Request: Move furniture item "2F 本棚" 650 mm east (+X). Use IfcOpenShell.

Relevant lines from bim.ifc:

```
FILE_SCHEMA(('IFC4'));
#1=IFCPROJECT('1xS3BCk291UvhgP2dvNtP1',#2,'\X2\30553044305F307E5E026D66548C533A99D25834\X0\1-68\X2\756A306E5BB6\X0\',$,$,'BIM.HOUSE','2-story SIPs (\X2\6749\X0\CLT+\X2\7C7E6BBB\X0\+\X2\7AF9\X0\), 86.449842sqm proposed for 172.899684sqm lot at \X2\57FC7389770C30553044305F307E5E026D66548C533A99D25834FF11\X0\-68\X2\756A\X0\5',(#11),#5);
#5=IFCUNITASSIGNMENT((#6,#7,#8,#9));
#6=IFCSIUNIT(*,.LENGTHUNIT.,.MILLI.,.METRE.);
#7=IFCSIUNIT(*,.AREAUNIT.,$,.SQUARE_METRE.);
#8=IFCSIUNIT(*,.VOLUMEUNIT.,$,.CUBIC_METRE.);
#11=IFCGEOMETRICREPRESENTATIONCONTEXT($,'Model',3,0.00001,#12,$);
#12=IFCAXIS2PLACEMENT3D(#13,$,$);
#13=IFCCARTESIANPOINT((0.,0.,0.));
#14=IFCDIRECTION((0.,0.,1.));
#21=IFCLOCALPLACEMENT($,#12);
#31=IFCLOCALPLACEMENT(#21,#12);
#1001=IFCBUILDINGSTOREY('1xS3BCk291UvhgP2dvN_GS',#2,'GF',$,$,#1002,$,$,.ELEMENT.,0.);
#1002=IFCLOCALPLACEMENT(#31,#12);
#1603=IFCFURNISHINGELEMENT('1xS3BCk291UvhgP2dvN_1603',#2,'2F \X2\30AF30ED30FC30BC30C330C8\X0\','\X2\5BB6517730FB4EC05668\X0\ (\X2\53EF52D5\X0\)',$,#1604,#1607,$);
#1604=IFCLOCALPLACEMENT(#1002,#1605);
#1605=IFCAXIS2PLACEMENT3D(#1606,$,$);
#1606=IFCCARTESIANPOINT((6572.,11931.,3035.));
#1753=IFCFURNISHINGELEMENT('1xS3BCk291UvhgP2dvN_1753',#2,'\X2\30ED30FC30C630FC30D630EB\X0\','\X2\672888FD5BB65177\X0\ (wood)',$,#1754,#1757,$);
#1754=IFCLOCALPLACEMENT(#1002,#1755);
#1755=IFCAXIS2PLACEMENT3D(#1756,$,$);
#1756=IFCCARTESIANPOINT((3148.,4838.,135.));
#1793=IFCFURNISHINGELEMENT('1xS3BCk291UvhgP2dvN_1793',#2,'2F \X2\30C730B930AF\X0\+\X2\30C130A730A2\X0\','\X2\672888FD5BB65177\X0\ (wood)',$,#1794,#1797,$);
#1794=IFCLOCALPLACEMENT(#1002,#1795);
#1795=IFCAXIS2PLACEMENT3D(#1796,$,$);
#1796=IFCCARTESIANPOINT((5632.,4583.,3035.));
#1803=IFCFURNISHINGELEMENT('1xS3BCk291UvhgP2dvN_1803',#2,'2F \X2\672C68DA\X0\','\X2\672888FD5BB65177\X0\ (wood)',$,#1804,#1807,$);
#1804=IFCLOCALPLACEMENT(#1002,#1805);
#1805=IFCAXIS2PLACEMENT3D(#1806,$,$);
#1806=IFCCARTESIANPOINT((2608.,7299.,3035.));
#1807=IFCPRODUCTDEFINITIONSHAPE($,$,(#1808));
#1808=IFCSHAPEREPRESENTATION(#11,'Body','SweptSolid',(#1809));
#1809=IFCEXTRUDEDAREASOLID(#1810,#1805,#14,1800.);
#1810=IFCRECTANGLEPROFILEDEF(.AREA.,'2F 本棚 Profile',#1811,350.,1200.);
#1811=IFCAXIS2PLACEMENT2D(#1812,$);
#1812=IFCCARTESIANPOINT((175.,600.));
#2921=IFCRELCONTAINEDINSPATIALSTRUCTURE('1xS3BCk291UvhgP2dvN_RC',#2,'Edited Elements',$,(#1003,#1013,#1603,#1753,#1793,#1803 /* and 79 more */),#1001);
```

```python
import ifcopenshell
import ifcopenshell.api.geometry
import ifcopenshell.util.placement

model = ifcopenshell.open("bim.ifc")

item = model.by_id(1803)
matrix = ifcopenshell.util.placement.get_local_placement(item.ObjectPlacement)
matrix[0, 3] += 650.0
ifcopenshell.api.geometry.edit_object_placement(model, product=item, matrix=matrix, is_si=False)

print(ifcopenshell.util.placement.get_local_placement(item.ObjectPlacement).round(3) + 0.0)

model.write("bim_v2.ifc")
```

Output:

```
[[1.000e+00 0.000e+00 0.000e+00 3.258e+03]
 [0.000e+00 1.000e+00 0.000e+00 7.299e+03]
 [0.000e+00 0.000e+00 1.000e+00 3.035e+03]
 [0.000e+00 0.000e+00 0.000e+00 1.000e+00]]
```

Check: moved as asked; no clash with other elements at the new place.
